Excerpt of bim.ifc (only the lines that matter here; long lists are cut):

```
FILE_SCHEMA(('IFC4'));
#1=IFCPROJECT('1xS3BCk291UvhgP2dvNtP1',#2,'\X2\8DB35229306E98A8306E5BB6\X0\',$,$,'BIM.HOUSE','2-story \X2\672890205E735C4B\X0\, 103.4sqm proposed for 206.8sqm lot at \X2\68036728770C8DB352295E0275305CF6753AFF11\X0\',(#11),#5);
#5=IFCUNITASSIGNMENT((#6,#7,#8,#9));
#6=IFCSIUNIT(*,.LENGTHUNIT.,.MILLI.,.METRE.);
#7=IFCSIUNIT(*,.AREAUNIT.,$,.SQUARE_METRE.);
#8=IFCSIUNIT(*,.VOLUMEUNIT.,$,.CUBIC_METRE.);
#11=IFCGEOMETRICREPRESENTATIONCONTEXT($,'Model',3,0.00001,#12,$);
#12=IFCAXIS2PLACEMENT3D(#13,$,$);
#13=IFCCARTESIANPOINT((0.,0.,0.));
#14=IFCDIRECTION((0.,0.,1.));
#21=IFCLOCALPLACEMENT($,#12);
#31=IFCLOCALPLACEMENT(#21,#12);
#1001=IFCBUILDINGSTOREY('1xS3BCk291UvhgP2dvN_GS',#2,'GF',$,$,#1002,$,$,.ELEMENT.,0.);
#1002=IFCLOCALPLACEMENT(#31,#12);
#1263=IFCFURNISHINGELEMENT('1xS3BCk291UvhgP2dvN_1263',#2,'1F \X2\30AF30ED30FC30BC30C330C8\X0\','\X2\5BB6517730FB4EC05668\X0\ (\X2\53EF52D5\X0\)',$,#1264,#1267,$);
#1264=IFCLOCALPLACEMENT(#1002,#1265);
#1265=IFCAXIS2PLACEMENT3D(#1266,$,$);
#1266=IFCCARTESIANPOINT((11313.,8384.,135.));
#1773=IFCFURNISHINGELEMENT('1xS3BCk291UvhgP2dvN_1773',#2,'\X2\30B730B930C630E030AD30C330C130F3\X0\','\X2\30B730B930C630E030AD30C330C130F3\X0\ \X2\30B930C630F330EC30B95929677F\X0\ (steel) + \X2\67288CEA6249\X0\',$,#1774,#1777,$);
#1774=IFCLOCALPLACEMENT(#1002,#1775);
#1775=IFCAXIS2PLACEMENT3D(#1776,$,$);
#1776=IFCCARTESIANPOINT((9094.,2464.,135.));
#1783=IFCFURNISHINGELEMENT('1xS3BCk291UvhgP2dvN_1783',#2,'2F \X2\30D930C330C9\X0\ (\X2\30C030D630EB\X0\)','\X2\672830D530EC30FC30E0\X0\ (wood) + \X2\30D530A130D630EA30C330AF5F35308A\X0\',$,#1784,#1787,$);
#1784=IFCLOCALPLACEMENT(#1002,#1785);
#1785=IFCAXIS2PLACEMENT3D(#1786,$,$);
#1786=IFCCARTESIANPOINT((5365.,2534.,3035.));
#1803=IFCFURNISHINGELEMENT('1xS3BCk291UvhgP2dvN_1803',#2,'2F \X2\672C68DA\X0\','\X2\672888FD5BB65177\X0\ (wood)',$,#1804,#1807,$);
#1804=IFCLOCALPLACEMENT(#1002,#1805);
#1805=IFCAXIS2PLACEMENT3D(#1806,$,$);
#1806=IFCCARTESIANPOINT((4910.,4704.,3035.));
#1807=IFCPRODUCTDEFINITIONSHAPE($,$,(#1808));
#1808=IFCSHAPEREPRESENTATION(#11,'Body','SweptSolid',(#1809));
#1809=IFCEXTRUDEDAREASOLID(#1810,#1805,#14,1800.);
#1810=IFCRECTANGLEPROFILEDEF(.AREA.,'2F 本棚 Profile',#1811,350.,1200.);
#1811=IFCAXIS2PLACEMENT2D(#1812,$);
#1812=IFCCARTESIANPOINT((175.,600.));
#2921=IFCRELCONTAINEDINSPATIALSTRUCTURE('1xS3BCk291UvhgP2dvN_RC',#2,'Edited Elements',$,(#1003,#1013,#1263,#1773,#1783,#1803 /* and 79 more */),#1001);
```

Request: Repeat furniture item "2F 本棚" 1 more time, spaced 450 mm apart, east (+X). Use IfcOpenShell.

```python
import numpy as np
import ifcopenshell
import ifcopenshell.api.geometry
import ifcopenshell.api.root
import ifcopenshell.util.element
import ifcopenshell.util.placement

model = ifcopenshell.open("bim.ifc")


def reuse_history(source, copy):
    """copy_class also copies each property set's owner history, people and application; keep the originals."""
    for rel in copy.IsDefinedBy:
        if rel.is_a("IfcRelDefinesByProperties") and (history := rel.RelatingPropertyDefinition.OwnerHistory):
            rel.RelatingPropertyDefinition.OwnerHistory = source.OwnerHistory
            ifcopenshell.util.element.remove_deep2(model, history)


source = model.by_guid("1xS3BCk291UvhgP2dvN_1803")
base = ifcopenshell.util.placement.get_local_placement(source.ObjectPlacement)
step = np.array([1.0, 0.0, 0.0]) * 450.0

for i in range(1, 2):
    copy = ifcopenshell.api.root.copy_class(model, product=source)
    copy.Representation = ifcopenshell.util.element.copy_deep(
        model, source.Representation, exclude=["IfcGeometricRepresentationContext", "IfcRepresentationMap"]
    )
    reuse_history(source, copy)
    matrix = base.copy()
    matrix[:3, 3] += i * step
    print("added at", matrix[:3, 3].round(3) + 0.0)
    ifcopenshell.api.geometry.edit_object_placement(model, product=copy, matrix=matrix, is_si=False)

model.write("bim_v2.ifc")
```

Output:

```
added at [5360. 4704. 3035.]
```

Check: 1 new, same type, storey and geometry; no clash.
